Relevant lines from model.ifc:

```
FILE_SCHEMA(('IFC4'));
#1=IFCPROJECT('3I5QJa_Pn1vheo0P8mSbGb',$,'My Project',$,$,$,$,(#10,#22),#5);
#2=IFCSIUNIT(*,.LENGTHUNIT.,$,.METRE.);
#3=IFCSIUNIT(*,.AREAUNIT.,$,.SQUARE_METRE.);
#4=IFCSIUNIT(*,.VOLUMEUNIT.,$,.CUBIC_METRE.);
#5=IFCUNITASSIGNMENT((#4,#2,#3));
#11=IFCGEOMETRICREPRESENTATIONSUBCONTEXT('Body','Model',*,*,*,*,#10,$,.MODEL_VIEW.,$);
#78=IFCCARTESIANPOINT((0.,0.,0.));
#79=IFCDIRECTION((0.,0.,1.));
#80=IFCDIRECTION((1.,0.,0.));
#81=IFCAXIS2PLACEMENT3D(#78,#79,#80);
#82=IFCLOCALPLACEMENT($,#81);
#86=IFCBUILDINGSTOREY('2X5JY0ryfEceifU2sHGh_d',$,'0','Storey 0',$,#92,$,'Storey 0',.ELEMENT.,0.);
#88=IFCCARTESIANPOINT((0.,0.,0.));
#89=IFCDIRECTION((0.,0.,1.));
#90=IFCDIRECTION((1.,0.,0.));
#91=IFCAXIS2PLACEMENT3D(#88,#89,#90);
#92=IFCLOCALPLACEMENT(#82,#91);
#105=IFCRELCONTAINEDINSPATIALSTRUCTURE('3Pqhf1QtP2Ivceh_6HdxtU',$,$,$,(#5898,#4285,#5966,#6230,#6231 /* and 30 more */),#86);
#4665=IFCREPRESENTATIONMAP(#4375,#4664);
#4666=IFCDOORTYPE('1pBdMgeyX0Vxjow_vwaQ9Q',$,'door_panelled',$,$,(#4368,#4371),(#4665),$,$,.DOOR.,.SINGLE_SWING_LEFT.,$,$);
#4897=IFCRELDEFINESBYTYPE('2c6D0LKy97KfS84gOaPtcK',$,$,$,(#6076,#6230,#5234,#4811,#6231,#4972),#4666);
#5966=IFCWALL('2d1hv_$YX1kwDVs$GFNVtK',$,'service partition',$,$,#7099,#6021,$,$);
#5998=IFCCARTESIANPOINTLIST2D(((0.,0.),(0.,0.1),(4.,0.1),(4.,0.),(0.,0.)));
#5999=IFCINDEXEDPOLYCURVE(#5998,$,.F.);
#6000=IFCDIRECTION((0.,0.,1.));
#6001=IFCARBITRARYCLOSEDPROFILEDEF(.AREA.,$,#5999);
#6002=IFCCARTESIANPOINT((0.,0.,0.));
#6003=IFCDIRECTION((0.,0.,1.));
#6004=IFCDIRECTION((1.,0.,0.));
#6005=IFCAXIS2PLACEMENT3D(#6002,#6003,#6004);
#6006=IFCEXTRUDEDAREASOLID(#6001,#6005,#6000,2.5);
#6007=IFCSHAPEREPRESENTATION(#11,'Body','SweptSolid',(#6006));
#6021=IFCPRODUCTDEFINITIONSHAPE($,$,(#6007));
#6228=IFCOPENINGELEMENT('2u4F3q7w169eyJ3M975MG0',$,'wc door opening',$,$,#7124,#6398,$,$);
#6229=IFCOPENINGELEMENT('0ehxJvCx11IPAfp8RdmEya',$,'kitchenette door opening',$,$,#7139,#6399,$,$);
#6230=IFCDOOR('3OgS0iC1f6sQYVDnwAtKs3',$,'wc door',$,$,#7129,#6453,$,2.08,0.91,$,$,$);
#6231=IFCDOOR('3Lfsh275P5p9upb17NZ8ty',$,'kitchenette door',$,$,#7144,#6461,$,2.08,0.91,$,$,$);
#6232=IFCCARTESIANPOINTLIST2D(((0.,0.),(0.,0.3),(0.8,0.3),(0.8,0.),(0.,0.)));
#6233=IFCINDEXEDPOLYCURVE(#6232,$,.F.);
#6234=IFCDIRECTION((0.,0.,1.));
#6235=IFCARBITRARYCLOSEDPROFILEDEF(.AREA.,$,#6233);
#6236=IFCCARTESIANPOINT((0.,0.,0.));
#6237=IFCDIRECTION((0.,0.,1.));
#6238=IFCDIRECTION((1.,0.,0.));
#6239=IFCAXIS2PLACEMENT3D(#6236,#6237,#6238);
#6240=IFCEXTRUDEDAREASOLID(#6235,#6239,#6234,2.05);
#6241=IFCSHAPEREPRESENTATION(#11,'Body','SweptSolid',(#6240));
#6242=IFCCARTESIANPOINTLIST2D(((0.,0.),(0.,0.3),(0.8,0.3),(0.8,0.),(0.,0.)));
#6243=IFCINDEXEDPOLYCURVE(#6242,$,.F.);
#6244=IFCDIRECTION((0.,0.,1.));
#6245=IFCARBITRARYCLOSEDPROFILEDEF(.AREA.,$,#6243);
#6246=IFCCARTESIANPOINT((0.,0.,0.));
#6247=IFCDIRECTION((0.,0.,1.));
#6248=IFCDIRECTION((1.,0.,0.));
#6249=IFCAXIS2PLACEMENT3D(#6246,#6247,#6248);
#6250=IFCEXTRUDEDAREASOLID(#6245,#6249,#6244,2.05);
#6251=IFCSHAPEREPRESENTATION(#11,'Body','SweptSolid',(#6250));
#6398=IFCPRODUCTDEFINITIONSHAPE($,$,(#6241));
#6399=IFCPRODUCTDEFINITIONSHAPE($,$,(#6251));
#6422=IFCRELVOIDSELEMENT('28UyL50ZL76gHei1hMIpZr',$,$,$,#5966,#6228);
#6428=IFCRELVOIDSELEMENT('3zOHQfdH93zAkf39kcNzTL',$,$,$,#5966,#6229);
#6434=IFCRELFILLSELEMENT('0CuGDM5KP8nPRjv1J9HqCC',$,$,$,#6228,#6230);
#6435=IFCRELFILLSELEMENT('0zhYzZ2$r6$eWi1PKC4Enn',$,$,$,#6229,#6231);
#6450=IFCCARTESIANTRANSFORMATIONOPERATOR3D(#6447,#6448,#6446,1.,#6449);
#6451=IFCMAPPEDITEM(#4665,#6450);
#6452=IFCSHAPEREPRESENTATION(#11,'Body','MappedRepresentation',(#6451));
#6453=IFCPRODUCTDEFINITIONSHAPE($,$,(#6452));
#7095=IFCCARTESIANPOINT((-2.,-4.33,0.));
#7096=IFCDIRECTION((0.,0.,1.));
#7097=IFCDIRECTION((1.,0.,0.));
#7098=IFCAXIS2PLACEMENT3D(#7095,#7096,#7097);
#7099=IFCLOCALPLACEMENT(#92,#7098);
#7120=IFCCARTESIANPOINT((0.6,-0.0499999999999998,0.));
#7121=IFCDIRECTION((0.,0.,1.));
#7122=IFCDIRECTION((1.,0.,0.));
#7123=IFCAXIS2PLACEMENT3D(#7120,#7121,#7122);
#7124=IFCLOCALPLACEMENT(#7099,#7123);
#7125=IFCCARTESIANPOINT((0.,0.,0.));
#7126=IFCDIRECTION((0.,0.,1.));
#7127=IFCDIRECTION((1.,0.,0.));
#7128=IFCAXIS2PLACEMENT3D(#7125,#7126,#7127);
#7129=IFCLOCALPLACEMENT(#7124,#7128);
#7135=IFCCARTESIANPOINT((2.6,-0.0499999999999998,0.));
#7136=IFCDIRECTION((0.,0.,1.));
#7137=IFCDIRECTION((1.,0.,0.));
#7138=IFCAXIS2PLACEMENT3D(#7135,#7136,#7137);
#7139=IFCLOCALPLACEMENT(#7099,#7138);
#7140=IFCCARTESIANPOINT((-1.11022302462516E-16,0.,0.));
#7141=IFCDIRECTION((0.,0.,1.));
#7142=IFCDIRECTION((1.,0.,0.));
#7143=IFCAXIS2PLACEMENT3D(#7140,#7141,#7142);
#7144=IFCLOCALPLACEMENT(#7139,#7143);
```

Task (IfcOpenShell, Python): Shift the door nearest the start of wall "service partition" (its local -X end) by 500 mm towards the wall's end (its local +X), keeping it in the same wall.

```python
import ifcopenshell
import ifcopenshell.api.geometry
import ifcopenshell.util.placement

model = ifcopenshell.open("model.ifc")

door = model.by_guid("3OgS0iC1f6sQYVDnwAtKs3")
opening = door.FillsVoids[0].RelatingOpeningElement
wall = opening.VoidsElements[0].RelatingBuildingElement

wall_matrix = ifcopenshell.util.placement.get_local_placement(wall.ObjectPlacement)
shift = wall_matrix[:3, 0] * 0.5
before = ifcopenshell.util.placement.get_local_placement(door.ObjectPlacement)[:3, 3].copy()

# The door is placed relative to its opening, so it follows when the opening moves.
matrix = ifcopenshell.util.placement.get_local_placement(opening.ObjectPlacement)
matrix[:3, 3] += shift
ifcopenshell.api.geometry.edit_object_placement(
    model, product=opening, matrix=matrix, is_si=False, should_transform_children=True
)

after = ifcopenshell.util.placement.get_local_placement(door.ObjectPlacement)[:3, 3]
print("door moved by", (after - before).round(3) + 0.0)

model.write("model-out.ifc")
```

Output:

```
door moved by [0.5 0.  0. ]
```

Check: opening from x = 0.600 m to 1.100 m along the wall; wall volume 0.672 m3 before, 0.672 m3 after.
